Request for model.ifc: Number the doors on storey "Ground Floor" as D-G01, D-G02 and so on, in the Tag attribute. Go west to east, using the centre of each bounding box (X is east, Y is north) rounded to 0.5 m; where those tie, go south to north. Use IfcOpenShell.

First a look at what the model holds.

```python
import ifcopenshell
import ifcopenshell.util.element
import ifcopenshell.util.placement

model = ifcopenshell.open("model.ifc")
print(model.schema)
storey = next(s for s in model.by_type("IfcBuildingStorey") if s.Name == "Ground Floor")
doors = [e for e in ifcopenshell.util.element.get_decomposition(storey) if e.is_a("IfcDoor")]
for e in sorted(doors, key=lambda e: e.id()):
    origin = ifcopenshell.util.placement.get_local_placement(e.ObjectPlacement)[:3, 3]
    print(e.id(), e.Tag, e.Name, origin.round(2) + 0.0, sep=" | ")
```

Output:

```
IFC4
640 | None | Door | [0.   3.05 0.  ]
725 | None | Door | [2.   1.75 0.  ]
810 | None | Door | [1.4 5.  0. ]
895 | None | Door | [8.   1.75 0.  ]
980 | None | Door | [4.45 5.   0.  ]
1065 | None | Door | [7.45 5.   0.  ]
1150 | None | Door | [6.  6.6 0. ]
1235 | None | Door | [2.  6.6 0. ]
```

```python
import ifcopenshell
import ifcopenshell.geom
import ifcopenshell.util.element
import ifcopenshell.util.shape

model = ifcopenshell.open("model.ifc")
settings = ifcopenshell.geom.settings()
settings.set("use-world-coords", True)


def centre(element):
    shape = ifcopenshell.geom.create_shape(settings, element)
    return ifcopenshell.util.shape.get_bbox_centroid(shape.geometry)


storey = next(s for s in model.by_type("IfcBuildingStorey") if s.Name == "Ground Floor")
doors = [e for e in ifcopenshell.util.element.get_decomposition(storey) if e.is_a("IfcDoor")]

# Insertion points can sit at a corner or the storey origin, so sort by the geometry (in metres).
centres = {e: centre(e) for e in doors}
doors.sort(key=lambda e: (round(centres[e][0] / 0.5), centres[e][1]))

for i, e in enumerate(doors, start=1):
    number = f"D-G{i:02d}"
    e.Tag = number
    print(e.id(), number)

model.write("model-out.ifc")
```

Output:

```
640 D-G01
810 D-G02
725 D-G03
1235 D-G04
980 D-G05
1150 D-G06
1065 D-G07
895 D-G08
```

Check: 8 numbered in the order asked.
